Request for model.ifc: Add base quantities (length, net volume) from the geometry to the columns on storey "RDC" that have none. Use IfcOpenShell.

First a look at what the model holds.

```python
import ifcopenshell
import ifcopenshell.util.element
import ifcopenshell.util.unit

model = ifcopenshell.open("model.ifc")
print(model.schema)
for unit_type in ("LENGTHUNIT", "AREAUNIT", "VOLUMEUNIT"):
    print(unit_type, ifcopenshell.util.unit.calculate_unit_scale(model, unit_type))
storey = next(s for s in model.by_type("IfcBuildingStorey") if s.Name == "RDC")
columns = [e for e in ifcopenshell.util.element.get_decomposition(storey) if e.is_a("IfcColumn")]
for e in sorted(columns, key=lambda e: e.id()):
    print(e.id(), e.is_a(), e.Name, list(ifcopenshell.util.element.get_psets(e, qtos_only=True)), sep=" | ")
```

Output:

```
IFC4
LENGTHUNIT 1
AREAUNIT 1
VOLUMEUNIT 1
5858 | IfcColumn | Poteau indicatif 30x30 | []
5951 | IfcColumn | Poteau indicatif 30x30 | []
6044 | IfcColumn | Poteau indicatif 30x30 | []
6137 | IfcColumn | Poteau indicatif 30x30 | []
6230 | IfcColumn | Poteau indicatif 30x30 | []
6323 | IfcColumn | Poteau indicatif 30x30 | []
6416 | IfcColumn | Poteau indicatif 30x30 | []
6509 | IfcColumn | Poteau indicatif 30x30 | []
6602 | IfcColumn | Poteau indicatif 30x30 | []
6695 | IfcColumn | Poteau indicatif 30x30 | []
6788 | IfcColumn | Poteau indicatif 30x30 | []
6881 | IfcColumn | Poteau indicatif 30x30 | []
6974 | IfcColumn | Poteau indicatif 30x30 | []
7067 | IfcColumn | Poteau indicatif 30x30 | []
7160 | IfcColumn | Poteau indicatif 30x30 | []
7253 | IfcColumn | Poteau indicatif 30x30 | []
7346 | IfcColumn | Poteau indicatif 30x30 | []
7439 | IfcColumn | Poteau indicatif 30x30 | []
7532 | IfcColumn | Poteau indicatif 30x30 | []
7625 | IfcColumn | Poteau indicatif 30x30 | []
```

```python
import ifcopenshell
import ifcopenshell.api.pset
import ifcopenshell.geom
import ifcopenshell.util.element
import ifcopenshell.util.shape
import ifcopenshell.util.unit

model = ifcopenshell.open("model.ifc")
unit_scale = ifcopenshell.util.unit.calculate_unit_scale(model)
volume_scale = ifcopenshell.util.unit.calculate_unit_scale(model, "VOLUMEUNIT")
settings = ifcopenshell.geom.settings()

storey = next(s for s in model.by_type("IfcBuildingStorey") if s.Name == "RDC")
columns = [e for e in ifcopenshell.util.element.get_decomposition(storey) if e.is_a("IfcColumn")]

for e in sorted(columns, key=lambda e: e.id()):
    if ifcopenshell.util.element.get_psets(e, qtos_only=True, should_inherit=False):
        continue
    # Geometry comes back in metres, in the element's own axes.
    shape = ifcopenshell.geom.create_shape(settings, e)
    values = {
        "Length": ifcopenshell.util.shape.get_z(shape.geometry) / unit_scale,
        "NetVolume": ifcopenshell.util.shape.get_volume(shape.geometry) / volume_scale,
    }
    qto = ifcopenshell.api.pset.add_qto(model, product=e, name="Qto_ColumnBaseQuantities")
    ifcopenshell.api.pset.edit_qto(model, qto=qto, properties=values)
    print(e.id(), {k: round(v, 3) for k, v in values.items()})

model.write("model_v2.ifc")
```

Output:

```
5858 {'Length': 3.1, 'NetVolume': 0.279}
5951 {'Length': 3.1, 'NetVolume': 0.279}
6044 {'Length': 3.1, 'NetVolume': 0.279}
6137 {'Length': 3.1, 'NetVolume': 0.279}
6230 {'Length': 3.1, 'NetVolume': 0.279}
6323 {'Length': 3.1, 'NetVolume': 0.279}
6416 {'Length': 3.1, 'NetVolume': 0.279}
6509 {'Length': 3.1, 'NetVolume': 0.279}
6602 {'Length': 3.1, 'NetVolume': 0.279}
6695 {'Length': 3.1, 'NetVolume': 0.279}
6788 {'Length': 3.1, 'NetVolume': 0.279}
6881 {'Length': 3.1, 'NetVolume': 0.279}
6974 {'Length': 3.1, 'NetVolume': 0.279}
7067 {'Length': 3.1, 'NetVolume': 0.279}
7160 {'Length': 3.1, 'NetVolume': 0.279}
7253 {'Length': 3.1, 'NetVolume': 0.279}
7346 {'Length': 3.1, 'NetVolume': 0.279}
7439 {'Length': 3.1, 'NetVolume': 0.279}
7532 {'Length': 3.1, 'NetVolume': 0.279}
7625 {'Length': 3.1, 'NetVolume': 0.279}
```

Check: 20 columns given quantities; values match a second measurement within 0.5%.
